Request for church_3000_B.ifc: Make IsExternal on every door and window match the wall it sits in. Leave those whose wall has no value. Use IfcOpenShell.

First a look at what the model holds.

```python
import ifcopenshell
import ifcopenshell.util.element

model = ifcopenshell.open("church_3000_B.ifc")
print(model.schema)
seen = {}
for e in model.by_type("IfcDoor") + model.by_type("IfcWindow"):
    if not e.FillsVoids:
        continue
    host = e.FillsVoids[0].RelatingOpeningElement.VoidsElements[0].RelatingBuildingElement
    own = ifcopenshell.util.element.get_pset(e, f"Pset_{e.is_a()[3:].removesuffix('StandardCase')}Common", "IsExternal")
    wall = ifcopenshell.util.element.get_pset(host, "Pset_WallCommon", "IsExternal")
    seen[e.is_a(), own, wall] = seen.get((e.is_a(), own, wall), 0) + 1
for (cls, own, wall), count in sorted(seen.items(), key=str):
    print(count, cls, "IsExternal:", own, "| host wall:", wall)
```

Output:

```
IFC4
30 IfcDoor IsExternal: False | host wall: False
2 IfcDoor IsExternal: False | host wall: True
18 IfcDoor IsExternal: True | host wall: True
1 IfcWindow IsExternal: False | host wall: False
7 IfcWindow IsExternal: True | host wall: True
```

```python
import ifcopenshell
import ifcopenshell.api.pset
import ifcopenshell.util.element

model = ifcopenshell.open("church_3000_B.ifc")

count = 0
for ifc_class, pset_name in (("IfcDoor", "Pset_DoorCommon"), ("IfcWindow", "Pset_WindowCommon")):
    for e in model.by_type(ifc_class):
        if not e.FillsVoids:
            continue
        host = e.FillsVoids[0].RelatingOpeningElement.VoidsElements[0].RelatingBuildingElement
        external = ifcopenshell.util.element.get_pset(host, "Pset_WallCommon", "IsExternal")
        if external is None or ifcopenshell.util.element.get_pset(e, pset_name, "IsExternal") == external:
            continue
        pset = ifcopenshell.api.pset.add_pset(model, product=e, name=pset_name)
        ifcopenshell.api.pset.edit_pset(model, pset=pset, properties={"IsExternal": external})
        count += 1

print(count, "updated")

model.write("church_3000_B_v2.ifc")
```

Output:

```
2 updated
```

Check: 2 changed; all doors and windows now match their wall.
